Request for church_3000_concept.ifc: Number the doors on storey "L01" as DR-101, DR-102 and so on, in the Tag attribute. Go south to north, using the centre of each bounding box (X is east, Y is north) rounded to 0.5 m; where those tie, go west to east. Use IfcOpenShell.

First a look at what the model holds.

```python
import ifcopenshell
import ifcopenshell.util.element
import ifcopenshell.util.placement

model = ifcopenshell.open("church_3000_concept.ifc")
print(model.schema)
storey = next(s for s in model.by_type("IfcBuildingStorey") if s.Name == "L01")
doors = [e for e in ifcopenshell.util.element.get_decomposition(storey) if e.is_a("IfcDoor")]
for e in sorted(doors, key=lambda e: e.id()):
    origin = ifcopenshell.util.placement.get_local_placement(e.ObjectPlacement)[:3, 3]
    print(e.id(), e.Tag, e.Name, origin.round(2) + 0.0, sep=" | ")
```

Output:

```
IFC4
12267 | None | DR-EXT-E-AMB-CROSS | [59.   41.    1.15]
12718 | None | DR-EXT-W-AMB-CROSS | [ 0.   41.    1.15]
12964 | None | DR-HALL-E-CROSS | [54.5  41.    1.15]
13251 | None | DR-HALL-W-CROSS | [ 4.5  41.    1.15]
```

```python
import ifcopenshell
import ifcopenshell.geom
import ifcopenshell.util.element
import ifcopenshell.util.shape

model = ifcopenshell.open("church_3000_concept.ifc")
settings = ifcopenshell.geom.settings()
settings.set("use-world-coords", True)


def centre(element):
    shape = ifcopenshell.geom.create_shape(settings, element)
    return ifcopenshell.util.shape.get_bbox_centroid(shape.geometry)


storey = next(s for s in model.by_type("IfcBuildingStorey") if s.Name == "L01")
doors = [e for e in ifcopenshell.util.element.get_decomposition(storey) if e.is_a("IfcDoor")]

# Insertion points can sit at a corner or the storey origin, so sort by the geometry (in metres).
centres = {e: centre(e) for e in doors}
doors.sort(key=lambda e: (round(centres[e][1] / 0.5), centres[e][0]))

for i, e in enumerate(doors, start=1):
    number = f"DR-1{i:02d}"
    e.Tag = number
    print(e.id(), number)

model.write("church_3000_concept-out.ifc")
```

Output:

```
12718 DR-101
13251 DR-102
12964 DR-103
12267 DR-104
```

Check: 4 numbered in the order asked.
